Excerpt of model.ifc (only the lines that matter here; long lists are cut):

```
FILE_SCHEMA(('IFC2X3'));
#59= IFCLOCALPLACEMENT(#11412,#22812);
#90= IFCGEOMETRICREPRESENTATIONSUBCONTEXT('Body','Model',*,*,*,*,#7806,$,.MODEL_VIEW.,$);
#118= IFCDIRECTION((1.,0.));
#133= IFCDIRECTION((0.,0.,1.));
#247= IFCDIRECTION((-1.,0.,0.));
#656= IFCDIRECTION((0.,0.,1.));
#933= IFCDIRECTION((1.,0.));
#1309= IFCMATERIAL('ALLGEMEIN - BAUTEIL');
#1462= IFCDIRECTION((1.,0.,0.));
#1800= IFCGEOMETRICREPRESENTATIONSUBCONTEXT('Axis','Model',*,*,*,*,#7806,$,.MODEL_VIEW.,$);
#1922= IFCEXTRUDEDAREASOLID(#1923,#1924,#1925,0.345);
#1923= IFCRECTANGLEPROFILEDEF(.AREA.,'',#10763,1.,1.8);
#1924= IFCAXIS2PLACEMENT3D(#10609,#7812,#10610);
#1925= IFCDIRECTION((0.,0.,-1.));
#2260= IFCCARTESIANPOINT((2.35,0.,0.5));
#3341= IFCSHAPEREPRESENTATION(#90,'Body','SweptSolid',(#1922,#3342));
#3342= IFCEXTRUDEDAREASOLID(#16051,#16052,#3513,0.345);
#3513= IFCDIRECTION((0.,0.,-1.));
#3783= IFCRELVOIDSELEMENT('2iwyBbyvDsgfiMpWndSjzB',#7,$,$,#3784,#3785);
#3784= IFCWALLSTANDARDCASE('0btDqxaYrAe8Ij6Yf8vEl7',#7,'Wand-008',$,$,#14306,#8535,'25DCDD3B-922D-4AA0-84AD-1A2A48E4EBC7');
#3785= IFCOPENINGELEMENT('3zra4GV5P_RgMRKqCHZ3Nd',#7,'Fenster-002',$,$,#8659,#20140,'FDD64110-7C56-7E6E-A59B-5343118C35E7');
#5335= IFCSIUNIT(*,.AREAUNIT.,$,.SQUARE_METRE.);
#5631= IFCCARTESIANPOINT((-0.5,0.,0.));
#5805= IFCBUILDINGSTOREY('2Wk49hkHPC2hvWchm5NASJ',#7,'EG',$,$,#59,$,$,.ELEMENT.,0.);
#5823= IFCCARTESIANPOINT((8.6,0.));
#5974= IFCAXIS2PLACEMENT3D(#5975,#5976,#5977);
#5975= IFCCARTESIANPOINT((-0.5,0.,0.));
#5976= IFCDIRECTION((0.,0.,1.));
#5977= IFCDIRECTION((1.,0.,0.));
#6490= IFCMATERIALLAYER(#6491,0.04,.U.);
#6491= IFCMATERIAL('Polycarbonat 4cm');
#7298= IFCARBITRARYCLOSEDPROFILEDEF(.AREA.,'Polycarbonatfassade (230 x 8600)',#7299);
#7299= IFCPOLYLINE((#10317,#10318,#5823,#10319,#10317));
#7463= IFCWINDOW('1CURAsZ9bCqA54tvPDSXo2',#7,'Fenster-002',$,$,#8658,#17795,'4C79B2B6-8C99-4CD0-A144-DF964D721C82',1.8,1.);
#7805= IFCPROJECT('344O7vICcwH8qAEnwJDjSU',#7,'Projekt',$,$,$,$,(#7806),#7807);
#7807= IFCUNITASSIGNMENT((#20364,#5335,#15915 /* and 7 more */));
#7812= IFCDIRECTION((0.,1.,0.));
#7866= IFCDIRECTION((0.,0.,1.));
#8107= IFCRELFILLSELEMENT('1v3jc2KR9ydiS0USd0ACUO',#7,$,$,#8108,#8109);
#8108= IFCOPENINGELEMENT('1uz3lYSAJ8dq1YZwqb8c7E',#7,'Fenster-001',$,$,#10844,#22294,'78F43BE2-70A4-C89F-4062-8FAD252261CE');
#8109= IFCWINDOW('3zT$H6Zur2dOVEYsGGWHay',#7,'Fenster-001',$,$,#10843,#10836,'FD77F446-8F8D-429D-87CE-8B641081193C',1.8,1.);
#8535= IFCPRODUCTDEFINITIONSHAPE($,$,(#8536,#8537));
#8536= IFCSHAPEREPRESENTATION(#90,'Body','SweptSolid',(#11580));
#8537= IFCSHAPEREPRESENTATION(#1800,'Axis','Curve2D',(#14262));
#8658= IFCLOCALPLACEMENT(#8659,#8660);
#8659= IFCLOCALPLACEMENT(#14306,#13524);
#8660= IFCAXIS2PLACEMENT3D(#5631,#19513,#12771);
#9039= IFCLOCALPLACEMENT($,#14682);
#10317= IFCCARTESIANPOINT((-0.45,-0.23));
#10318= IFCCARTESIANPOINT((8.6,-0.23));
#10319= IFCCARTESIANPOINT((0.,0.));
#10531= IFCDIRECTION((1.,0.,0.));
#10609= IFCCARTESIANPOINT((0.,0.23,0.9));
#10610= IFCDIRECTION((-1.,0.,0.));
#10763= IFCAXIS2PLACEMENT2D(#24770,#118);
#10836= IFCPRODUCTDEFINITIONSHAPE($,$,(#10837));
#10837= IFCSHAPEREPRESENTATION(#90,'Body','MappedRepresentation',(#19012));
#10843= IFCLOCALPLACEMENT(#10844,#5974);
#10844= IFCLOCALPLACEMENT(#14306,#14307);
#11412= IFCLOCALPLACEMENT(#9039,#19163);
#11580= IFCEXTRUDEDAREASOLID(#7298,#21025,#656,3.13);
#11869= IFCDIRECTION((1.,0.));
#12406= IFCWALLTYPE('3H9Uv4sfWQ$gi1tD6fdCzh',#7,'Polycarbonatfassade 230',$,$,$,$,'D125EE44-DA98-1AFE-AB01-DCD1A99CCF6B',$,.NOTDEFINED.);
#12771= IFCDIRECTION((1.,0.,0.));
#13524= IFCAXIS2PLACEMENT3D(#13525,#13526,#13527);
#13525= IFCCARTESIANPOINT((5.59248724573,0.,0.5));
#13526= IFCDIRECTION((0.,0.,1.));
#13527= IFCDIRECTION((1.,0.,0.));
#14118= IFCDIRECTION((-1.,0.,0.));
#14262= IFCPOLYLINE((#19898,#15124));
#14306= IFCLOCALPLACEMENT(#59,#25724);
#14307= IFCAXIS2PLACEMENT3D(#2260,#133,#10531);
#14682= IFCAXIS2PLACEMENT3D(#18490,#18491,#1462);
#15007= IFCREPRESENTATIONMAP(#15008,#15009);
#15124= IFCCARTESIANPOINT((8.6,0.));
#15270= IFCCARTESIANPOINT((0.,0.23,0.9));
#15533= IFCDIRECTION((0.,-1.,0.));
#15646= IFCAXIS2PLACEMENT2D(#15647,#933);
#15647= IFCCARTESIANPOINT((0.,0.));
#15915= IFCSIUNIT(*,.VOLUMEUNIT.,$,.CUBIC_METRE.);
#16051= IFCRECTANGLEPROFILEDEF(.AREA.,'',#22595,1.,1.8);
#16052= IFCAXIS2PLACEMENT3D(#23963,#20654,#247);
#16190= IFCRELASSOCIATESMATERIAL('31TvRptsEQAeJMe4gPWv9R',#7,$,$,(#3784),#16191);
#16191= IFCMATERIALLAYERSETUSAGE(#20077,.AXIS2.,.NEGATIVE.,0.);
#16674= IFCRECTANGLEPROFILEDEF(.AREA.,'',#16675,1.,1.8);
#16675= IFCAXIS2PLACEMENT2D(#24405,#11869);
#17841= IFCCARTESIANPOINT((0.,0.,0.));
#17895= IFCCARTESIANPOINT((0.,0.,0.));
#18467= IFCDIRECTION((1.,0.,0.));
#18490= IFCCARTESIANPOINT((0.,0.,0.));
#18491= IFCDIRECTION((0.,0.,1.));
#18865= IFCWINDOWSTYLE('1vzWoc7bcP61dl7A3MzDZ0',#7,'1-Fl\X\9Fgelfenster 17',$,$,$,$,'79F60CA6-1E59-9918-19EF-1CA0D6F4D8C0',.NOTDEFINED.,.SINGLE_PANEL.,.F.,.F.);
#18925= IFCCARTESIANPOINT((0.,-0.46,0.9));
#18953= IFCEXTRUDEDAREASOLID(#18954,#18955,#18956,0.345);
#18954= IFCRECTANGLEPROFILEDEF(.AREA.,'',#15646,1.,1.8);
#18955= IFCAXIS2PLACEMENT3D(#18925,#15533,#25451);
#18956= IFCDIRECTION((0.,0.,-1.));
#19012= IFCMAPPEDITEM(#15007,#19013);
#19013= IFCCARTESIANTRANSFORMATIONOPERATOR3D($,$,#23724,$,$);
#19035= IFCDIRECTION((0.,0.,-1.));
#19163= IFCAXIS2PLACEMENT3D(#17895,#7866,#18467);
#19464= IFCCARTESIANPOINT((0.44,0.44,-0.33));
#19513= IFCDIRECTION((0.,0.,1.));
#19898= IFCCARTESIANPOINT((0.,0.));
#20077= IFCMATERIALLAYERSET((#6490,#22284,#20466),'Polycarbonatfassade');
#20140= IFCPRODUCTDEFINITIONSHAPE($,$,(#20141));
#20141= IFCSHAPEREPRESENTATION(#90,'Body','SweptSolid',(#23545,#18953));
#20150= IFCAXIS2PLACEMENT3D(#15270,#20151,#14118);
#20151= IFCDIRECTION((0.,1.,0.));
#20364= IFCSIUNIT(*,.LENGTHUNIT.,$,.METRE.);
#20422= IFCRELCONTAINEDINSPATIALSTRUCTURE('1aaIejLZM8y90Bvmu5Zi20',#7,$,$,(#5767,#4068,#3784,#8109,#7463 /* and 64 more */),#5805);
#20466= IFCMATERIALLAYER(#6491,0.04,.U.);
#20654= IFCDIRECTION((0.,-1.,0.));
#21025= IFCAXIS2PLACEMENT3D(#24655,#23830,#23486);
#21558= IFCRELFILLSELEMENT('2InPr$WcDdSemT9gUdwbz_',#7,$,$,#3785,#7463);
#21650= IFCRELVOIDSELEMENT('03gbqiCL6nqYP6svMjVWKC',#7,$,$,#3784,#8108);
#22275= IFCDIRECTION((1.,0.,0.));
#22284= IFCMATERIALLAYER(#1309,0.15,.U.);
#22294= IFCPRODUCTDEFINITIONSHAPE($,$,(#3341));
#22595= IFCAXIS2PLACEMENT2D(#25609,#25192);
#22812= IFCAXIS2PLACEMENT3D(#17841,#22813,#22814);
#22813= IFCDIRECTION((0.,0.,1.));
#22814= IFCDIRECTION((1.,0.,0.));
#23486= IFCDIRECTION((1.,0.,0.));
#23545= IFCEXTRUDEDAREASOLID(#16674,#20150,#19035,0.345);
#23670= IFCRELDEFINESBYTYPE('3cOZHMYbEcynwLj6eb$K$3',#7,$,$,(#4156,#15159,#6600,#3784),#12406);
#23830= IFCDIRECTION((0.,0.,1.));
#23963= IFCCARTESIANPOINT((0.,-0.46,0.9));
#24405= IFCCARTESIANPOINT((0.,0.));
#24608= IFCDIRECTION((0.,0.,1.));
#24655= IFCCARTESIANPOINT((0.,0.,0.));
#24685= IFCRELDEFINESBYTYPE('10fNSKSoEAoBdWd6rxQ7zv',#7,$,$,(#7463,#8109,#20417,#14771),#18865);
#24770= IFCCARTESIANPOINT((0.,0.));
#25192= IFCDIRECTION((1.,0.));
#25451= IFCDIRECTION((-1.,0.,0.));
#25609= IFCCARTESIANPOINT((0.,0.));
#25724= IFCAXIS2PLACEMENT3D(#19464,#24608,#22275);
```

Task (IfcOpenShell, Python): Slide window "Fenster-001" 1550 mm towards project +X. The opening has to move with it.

```python
import ifcopenshell
import ifcopenshell.api.geometry
import ifcopenshell.util.placement

model = ifcopenshell.open("model.ifc")

window = model.by_id(8109)
opening = window.FillsVoids[0].RelatingOpeningElement
wall = opening.VoidsElements[0].RelatingBuildingElement

wall_matrix = ifcopenshell.util.placement.get_local_placement(wall.ObjectPlacement)
shift = wall_matrix[:3, 0] * 1.55
before = ifcopenshell.util.placement.get_local_placement(window.ObjectPlacement)[:3, 3].copy()

# The window is placed relative to its opening, so it follows when the opening moves.
matrix = ifcopenshell.util.placement.get_local_placement(opening.ObjectPlacement)
matrix[:3, 3] += shift
ifcopenshell.api.geometry.edit_object_placement(
    model, product=opening, matrix=matrix, is_si=False, should_transform_children=True
)

after = ifcopenshell.util.placement.get_local_placement(window.ObjectPlacement)[:3, 3]
print("window moved by", (after - before).round(3) + 0.0)

model.write("model-out.ifc")
```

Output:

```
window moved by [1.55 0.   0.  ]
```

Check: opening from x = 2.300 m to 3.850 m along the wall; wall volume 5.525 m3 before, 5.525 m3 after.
